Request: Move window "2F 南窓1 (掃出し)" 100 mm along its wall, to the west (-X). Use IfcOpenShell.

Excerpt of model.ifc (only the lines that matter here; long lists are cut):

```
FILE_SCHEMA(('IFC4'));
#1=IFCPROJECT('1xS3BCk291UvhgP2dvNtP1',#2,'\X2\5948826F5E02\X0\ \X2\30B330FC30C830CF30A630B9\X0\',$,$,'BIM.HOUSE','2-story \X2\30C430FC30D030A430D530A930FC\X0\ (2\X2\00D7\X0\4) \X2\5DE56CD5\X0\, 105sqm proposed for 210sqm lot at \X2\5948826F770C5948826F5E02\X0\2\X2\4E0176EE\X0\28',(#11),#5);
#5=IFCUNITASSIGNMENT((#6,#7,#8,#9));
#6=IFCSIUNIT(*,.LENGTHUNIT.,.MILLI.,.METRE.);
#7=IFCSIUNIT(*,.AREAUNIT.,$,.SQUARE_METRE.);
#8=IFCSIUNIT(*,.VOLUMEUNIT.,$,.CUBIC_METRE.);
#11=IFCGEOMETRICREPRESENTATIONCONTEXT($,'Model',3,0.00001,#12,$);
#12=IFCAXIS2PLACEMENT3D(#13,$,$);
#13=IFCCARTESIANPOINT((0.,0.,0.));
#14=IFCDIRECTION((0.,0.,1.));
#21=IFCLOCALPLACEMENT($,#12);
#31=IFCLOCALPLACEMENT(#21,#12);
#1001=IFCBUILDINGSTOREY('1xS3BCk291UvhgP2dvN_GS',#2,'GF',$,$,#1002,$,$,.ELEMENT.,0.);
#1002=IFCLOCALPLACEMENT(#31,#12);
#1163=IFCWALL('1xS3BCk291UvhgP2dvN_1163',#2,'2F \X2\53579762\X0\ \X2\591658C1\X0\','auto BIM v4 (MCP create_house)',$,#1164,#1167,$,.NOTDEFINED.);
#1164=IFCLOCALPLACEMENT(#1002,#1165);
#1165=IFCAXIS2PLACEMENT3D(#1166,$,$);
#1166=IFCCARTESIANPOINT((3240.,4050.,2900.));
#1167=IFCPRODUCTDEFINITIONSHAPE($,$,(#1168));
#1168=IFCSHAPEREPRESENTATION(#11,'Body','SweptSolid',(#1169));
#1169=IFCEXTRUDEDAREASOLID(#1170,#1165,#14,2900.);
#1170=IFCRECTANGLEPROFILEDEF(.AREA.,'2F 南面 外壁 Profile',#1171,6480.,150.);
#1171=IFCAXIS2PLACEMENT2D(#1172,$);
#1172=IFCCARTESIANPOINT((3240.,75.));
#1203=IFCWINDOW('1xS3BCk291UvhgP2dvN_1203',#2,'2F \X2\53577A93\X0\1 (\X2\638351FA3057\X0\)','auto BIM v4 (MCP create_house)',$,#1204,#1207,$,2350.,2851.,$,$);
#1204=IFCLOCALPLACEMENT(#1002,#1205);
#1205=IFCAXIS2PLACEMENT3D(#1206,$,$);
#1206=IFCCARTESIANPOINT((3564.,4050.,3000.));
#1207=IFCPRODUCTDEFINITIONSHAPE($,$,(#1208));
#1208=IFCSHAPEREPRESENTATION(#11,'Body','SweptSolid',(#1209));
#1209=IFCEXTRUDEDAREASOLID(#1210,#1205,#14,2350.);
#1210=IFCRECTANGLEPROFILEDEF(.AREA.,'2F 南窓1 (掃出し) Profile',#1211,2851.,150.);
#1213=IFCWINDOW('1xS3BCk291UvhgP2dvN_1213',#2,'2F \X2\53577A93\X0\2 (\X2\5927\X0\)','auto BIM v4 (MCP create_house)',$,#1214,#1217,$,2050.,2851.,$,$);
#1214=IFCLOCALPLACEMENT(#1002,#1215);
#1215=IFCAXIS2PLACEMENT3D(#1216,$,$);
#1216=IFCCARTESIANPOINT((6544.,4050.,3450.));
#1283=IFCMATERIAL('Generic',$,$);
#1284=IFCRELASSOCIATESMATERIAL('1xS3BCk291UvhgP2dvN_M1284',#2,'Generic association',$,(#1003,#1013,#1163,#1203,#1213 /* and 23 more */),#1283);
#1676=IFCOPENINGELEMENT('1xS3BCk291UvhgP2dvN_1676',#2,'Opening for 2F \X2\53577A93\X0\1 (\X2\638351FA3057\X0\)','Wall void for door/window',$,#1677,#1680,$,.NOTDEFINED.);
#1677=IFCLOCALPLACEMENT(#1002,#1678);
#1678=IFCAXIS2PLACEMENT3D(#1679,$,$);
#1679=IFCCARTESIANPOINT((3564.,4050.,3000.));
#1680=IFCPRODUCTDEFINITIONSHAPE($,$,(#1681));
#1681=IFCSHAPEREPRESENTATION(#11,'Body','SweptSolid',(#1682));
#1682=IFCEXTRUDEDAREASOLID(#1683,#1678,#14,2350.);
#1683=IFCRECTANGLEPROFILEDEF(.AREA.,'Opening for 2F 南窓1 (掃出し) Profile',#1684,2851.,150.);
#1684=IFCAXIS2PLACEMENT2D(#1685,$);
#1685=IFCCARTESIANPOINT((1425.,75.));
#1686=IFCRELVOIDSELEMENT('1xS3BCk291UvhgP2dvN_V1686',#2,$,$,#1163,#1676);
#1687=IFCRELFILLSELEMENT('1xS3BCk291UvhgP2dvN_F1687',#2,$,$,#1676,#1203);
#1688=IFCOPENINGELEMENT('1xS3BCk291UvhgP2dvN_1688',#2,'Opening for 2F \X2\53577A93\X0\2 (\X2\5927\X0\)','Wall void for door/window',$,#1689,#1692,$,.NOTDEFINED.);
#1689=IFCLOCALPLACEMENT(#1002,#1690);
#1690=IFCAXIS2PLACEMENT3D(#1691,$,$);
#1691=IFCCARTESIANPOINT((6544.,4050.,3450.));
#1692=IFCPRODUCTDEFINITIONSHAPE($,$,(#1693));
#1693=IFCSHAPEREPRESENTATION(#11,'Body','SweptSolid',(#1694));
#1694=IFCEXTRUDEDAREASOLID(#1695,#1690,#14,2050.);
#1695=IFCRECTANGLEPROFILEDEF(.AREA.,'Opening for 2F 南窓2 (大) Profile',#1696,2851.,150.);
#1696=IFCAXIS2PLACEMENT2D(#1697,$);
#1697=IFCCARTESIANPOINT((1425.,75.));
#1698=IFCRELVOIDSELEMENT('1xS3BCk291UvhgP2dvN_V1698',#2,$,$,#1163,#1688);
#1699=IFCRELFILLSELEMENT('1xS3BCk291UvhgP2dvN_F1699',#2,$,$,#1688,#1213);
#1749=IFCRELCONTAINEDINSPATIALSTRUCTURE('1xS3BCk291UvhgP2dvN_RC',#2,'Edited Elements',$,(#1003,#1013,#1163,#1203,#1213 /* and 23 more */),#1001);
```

```python
import ifcopenshell
import ifcopenshell.api.geometry
import ifcopenshell.util.placement
import ifcopenshell.util.unit

model = ifcopenshell.open("model.ifc")
unit_scale = ifcopenshell.util.unit.calculate_unit_scale(model)

window = model.by_guid("1xS3BCk291UvhgP2dvN_1203")
opening = window.FillsVoids[0].RelatingOpeningElement
wall = opening.VoidsElements[0].RelatingBuildingElement

wall_matrix = ifcopenshell.util.placement.get_local_placement(wall.ObjectPlacement)
shift = wall_matrix[:3, 0] * -0.1 / unit_scale
before = ifcopenshell.util.placement.get_local_placement(window.ObjectPlacement)[:3, 3].copy()

# The window is not placed relative to its opening, so move both.
for product in (opening, window):
    matrix = ifcopenshell.util.placement.get_local_placement(product.ObjectPlacement)
    matrix[:3, 3] += shift
    ifcopenshell.api.geometry.edit_object_placement(model, product=product, matrix=matrix, is_si=False)

after = ifcopenshell.util.placement.get_local_placement(window.ObjectPlacement)[:3, 3]
print("window moved by", (after - before).round(3) + 0.0)

model.write("model_v2.ifc")
```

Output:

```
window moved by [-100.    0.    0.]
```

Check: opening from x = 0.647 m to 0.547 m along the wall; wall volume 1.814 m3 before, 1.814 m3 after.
